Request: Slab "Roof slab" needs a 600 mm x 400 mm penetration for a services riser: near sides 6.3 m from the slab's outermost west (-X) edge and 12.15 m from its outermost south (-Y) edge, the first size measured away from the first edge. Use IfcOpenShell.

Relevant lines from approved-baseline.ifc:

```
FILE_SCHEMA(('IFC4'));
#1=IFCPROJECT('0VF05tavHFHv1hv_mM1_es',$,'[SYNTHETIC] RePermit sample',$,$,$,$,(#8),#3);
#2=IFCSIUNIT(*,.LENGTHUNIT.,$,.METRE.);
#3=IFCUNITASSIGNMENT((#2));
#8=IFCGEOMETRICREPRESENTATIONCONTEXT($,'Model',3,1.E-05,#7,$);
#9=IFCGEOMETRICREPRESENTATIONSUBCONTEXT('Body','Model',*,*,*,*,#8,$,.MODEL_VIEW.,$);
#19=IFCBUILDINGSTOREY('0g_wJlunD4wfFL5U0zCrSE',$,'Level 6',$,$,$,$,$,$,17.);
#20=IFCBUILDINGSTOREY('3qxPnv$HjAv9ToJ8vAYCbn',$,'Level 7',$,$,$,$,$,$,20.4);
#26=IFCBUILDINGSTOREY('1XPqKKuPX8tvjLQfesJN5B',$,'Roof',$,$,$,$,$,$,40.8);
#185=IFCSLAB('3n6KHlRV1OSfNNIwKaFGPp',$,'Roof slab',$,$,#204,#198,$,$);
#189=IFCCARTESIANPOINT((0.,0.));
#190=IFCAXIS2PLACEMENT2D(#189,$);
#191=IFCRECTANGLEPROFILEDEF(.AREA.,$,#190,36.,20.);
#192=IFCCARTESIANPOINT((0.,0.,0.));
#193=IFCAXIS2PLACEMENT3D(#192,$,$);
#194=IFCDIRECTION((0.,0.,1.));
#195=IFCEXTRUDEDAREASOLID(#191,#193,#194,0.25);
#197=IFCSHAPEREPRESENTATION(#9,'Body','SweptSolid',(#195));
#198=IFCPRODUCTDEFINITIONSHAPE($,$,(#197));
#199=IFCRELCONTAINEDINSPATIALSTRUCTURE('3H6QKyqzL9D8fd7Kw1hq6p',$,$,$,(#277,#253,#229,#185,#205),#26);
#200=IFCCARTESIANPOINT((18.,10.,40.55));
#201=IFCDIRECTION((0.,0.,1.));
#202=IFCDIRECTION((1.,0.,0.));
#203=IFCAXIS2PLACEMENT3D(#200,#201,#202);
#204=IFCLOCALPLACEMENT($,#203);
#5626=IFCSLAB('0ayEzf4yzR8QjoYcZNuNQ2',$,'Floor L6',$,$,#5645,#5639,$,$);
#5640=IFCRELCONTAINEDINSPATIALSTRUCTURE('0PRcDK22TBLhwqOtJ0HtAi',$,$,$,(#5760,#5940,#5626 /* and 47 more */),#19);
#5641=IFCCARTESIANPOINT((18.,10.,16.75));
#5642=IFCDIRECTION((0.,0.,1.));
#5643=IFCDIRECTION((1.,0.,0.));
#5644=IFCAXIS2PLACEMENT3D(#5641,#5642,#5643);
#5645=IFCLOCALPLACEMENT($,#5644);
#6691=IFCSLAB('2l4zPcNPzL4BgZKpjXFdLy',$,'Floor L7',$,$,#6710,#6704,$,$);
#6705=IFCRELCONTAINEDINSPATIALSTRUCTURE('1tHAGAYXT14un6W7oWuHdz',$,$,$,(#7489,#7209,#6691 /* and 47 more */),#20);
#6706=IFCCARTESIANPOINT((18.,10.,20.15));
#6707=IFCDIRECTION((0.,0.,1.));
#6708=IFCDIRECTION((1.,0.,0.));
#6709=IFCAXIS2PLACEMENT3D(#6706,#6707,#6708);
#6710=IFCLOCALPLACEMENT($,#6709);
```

```python
import numpy as np
import ifcopenshell
import ifcopenshell.api.feature
import ifcopenshell.api.geometry
import ifcopenshell.api.root
import ifcopenshell.geom
import ifcopenshell.util.placement
import ifcopenshell.util.representation
import ifcopenshell.util.shape
import ifcopenshell.util.unit

model = ifcopenshell.open("approved-baseline.ifc")
unit_scale = ifcopenshell.util.unit.calculate_unit_scale(model)
settings = ifcopenshell.geom.settings()


def volume(element):
    """Net volume in cubic metres, openings subtracted."""
    shape = ifcopenshell.geom.create_shape(settings, element)
    return ifcopenshell.util.shape.get_volume(shape.geometry)


slab = model.by_id(185)
before = volume(slab)

# Extent in the slab's own axes, in metres. The edges named are its -X and -Y sides.
slab_shape = ifcopenshell.geom.create_shape(settings, slab)
vertices = ifcopenshell.util.shape.get_vertices(slab_shape.geometry)
x_min, y_min, bottom = vertices.min(axis=0)
top = vertices[:, 2].max()

opening = ifcopenshell.api.root.create_entity(model, ifc_class="IfcOpeningElement", name="Services riser opening", predefined_type="OPENING")
context = ifcopenshell.util.representation.get_context(model, "Model", "Body", "MODEL_VIEW")
width, depth = 0.6, 0.4
outline = [(0.0, 0.0), (width, 0.0), (width, depth), (0.0, depth), (0.0, 0.0)]
# Overshoot both faces by 50 mm so the cut is clean.
shape = ifcopenshell.api.geometry.add_slab_representation(
    model, context=context, depth=top - bottom + 0.1, polyline=outline
)
ifcopenshell.api.geometry.assign_representation(model, product=opening, representation=shape)

matrix = ifcopenshell.util.placement.get_local_placement(slab.ObjectPlacement)
matrix[:, 3] = matrix @ np.append(np.array([x_min + 6.3, y_min + 12.15, bottom - 0.05]) / unit_scale, 1.0)
ifcopenshell.api.geometry.edit_object_placement(model, product=opening, matrix=matrix, is_si=False)
ifcopenshell.api.feature.add_feature(model, feature=opening, element=slab)

after = volume(slab)

print(f"slab volume {before:.3f} -> {after:.3f} m3")

model.write("approved-baseline_v2.ifc")
```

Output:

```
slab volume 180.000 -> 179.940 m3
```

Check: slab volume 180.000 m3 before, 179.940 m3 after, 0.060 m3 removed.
